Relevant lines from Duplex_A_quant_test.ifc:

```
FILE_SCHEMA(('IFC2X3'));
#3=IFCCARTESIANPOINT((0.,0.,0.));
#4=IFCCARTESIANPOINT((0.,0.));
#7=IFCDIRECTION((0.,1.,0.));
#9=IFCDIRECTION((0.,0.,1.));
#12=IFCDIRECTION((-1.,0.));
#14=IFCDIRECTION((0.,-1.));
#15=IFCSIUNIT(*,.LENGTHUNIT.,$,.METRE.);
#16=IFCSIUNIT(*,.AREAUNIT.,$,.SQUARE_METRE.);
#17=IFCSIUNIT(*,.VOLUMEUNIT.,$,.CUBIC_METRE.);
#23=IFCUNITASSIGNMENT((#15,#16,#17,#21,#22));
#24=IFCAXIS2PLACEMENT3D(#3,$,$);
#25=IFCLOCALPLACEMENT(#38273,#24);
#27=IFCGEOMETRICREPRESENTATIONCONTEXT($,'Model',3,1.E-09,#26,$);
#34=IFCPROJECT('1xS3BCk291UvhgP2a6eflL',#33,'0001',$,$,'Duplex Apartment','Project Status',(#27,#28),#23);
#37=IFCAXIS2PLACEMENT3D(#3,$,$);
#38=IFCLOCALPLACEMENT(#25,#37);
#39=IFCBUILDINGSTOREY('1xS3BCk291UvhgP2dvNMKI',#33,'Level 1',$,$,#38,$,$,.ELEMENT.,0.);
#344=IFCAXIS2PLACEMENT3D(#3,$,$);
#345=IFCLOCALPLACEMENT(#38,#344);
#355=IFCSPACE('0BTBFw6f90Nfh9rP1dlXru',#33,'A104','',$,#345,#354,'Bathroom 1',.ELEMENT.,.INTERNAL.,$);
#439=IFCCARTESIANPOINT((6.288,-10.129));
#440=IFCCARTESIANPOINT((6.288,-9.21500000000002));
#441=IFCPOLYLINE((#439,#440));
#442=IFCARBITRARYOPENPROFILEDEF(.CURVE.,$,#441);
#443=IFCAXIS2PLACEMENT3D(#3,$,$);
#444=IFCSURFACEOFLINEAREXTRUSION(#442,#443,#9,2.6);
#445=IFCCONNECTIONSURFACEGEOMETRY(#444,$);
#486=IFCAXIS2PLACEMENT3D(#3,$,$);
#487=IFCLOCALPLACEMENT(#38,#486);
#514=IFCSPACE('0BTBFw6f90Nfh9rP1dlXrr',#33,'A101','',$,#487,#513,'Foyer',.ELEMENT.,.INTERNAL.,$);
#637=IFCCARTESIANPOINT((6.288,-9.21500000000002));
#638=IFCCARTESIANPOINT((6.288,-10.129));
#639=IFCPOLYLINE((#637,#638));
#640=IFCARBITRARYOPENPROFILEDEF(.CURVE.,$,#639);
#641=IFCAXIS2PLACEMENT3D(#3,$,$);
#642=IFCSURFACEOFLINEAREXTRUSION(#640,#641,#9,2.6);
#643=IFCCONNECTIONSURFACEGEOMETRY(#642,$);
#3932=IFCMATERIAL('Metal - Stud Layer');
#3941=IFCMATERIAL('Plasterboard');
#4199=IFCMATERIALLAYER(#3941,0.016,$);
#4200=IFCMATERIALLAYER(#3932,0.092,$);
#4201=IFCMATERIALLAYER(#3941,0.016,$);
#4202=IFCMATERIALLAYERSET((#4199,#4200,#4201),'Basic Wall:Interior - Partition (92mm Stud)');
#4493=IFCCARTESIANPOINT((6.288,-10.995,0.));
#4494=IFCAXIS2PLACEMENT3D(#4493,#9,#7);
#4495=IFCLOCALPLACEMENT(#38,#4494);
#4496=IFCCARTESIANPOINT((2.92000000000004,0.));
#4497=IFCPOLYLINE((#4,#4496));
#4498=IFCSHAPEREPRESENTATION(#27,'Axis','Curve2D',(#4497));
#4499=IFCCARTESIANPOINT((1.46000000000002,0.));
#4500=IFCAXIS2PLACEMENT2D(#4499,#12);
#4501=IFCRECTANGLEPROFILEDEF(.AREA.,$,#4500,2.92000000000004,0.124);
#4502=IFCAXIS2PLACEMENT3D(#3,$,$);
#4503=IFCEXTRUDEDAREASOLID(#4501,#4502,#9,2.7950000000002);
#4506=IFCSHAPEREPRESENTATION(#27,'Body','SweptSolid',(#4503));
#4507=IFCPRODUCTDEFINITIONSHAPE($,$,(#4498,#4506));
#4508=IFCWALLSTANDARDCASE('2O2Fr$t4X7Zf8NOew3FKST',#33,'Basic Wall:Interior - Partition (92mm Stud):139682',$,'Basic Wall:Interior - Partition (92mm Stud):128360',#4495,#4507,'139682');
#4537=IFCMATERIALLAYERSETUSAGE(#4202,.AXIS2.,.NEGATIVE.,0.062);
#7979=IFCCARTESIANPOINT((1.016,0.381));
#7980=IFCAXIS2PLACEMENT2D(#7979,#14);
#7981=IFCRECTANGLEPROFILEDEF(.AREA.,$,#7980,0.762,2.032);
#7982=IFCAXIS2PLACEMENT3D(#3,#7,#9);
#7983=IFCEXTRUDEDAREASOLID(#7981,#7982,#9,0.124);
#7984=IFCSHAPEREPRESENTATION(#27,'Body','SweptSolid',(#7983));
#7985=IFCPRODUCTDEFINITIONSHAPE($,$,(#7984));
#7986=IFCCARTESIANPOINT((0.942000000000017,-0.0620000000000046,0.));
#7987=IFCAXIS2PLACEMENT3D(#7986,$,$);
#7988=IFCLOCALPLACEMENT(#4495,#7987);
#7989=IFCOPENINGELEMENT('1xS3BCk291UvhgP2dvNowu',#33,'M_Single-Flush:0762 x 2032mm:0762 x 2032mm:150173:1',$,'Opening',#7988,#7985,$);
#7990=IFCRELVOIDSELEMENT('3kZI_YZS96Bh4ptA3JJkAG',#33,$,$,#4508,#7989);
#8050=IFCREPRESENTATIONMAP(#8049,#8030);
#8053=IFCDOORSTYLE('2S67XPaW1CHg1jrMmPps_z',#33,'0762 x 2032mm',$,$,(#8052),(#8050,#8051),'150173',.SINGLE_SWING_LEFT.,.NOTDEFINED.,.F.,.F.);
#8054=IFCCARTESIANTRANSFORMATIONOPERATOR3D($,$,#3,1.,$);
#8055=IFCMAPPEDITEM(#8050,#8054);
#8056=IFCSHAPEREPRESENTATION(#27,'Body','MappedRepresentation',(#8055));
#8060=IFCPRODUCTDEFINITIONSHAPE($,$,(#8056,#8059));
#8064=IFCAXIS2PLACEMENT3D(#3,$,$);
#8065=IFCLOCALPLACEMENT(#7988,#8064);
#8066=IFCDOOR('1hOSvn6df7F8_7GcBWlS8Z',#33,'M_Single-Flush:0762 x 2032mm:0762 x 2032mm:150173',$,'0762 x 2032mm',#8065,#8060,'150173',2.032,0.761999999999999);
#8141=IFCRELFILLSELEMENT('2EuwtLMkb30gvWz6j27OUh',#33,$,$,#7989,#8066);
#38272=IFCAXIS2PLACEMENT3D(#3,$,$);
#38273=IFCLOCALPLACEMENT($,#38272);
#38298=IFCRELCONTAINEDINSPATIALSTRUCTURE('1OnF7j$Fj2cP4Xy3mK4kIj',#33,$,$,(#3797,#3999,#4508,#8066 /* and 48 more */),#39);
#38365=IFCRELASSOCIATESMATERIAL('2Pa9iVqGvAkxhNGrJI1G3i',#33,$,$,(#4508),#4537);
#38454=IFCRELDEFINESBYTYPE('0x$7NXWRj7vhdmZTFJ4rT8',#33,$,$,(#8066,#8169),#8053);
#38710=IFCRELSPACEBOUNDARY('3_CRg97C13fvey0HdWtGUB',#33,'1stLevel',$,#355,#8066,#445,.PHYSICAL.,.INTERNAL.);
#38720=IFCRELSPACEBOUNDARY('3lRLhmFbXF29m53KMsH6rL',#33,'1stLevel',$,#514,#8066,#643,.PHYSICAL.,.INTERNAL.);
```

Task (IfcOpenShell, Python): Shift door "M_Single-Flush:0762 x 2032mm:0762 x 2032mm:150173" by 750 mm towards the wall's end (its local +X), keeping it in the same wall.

```python
import numpy as np
import ifcopenshell
import ifcopenshell.api.geometry
import ifcopenshell.util.placement

model = ifcopenshell.open("Duplex_A_quant_test.ifc")

door = model.by_guid("1hOSvn6df7F8_7GcBWlS8Z")
opening = door.FillsVoids[0].RelatingOpeningElement
wall = opening.VoidsElements[0].RelatingBuildingElement

wall_matrix = ifcopenshell.util.placement.get_local_placement(wall.ObjectPlacement)
shift = wall_matrix[:3, 0] * 0.75
before = ifcopenshell.util.placement.get_local_placement(door.ObjectPlacement)[:3, 3].copy()

# The door is placed relative to its opening, so it follows when the opening moves.
matrix = ifcopenshell.util.placement.get_local_placement(opening.ObjectPlacement)
matrix[:3, 3] += shift
ifcopenshell.api.geometry.edit_object_placement(
    model, product=opening, matrix=matrix, is_si=False, should_transform_children=True
)

# Space boundary surfaces are stored in each space's coordinates; move them too.
for rel in door.ProvidesBoundaries:
    if not rel.ConnectionGeometry:
        continue
    surface = rel.ConnectionGeometry.SurfaceOnRelatingElement
    space_matrix = ifcopenshell.util.placement.get_local_placement(rel.RelatingSpace.ObjectPlacement)
    point = np.array(surface.Position.Location.Coordinates) + space_matrix[:3, :3].T @ shift
    surface.Position = model.createIfcAxis2Placement3D(
        model.createIfcCartesianPoint(point.tolist()), surface.Position.Axis, surface.Position.RefDirection
    )

after = ifcopenshell.util.placement.get_local_placement(door.ObjectPlacement)[:3, 3]
print("door moved by", (after - before).round(3) + 0.0)

model.write("Duplex_A_quant_test_rev.ifc")
```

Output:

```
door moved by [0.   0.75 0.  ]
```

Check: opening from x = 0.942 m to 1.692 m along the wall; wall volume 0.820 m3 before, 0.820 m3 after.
